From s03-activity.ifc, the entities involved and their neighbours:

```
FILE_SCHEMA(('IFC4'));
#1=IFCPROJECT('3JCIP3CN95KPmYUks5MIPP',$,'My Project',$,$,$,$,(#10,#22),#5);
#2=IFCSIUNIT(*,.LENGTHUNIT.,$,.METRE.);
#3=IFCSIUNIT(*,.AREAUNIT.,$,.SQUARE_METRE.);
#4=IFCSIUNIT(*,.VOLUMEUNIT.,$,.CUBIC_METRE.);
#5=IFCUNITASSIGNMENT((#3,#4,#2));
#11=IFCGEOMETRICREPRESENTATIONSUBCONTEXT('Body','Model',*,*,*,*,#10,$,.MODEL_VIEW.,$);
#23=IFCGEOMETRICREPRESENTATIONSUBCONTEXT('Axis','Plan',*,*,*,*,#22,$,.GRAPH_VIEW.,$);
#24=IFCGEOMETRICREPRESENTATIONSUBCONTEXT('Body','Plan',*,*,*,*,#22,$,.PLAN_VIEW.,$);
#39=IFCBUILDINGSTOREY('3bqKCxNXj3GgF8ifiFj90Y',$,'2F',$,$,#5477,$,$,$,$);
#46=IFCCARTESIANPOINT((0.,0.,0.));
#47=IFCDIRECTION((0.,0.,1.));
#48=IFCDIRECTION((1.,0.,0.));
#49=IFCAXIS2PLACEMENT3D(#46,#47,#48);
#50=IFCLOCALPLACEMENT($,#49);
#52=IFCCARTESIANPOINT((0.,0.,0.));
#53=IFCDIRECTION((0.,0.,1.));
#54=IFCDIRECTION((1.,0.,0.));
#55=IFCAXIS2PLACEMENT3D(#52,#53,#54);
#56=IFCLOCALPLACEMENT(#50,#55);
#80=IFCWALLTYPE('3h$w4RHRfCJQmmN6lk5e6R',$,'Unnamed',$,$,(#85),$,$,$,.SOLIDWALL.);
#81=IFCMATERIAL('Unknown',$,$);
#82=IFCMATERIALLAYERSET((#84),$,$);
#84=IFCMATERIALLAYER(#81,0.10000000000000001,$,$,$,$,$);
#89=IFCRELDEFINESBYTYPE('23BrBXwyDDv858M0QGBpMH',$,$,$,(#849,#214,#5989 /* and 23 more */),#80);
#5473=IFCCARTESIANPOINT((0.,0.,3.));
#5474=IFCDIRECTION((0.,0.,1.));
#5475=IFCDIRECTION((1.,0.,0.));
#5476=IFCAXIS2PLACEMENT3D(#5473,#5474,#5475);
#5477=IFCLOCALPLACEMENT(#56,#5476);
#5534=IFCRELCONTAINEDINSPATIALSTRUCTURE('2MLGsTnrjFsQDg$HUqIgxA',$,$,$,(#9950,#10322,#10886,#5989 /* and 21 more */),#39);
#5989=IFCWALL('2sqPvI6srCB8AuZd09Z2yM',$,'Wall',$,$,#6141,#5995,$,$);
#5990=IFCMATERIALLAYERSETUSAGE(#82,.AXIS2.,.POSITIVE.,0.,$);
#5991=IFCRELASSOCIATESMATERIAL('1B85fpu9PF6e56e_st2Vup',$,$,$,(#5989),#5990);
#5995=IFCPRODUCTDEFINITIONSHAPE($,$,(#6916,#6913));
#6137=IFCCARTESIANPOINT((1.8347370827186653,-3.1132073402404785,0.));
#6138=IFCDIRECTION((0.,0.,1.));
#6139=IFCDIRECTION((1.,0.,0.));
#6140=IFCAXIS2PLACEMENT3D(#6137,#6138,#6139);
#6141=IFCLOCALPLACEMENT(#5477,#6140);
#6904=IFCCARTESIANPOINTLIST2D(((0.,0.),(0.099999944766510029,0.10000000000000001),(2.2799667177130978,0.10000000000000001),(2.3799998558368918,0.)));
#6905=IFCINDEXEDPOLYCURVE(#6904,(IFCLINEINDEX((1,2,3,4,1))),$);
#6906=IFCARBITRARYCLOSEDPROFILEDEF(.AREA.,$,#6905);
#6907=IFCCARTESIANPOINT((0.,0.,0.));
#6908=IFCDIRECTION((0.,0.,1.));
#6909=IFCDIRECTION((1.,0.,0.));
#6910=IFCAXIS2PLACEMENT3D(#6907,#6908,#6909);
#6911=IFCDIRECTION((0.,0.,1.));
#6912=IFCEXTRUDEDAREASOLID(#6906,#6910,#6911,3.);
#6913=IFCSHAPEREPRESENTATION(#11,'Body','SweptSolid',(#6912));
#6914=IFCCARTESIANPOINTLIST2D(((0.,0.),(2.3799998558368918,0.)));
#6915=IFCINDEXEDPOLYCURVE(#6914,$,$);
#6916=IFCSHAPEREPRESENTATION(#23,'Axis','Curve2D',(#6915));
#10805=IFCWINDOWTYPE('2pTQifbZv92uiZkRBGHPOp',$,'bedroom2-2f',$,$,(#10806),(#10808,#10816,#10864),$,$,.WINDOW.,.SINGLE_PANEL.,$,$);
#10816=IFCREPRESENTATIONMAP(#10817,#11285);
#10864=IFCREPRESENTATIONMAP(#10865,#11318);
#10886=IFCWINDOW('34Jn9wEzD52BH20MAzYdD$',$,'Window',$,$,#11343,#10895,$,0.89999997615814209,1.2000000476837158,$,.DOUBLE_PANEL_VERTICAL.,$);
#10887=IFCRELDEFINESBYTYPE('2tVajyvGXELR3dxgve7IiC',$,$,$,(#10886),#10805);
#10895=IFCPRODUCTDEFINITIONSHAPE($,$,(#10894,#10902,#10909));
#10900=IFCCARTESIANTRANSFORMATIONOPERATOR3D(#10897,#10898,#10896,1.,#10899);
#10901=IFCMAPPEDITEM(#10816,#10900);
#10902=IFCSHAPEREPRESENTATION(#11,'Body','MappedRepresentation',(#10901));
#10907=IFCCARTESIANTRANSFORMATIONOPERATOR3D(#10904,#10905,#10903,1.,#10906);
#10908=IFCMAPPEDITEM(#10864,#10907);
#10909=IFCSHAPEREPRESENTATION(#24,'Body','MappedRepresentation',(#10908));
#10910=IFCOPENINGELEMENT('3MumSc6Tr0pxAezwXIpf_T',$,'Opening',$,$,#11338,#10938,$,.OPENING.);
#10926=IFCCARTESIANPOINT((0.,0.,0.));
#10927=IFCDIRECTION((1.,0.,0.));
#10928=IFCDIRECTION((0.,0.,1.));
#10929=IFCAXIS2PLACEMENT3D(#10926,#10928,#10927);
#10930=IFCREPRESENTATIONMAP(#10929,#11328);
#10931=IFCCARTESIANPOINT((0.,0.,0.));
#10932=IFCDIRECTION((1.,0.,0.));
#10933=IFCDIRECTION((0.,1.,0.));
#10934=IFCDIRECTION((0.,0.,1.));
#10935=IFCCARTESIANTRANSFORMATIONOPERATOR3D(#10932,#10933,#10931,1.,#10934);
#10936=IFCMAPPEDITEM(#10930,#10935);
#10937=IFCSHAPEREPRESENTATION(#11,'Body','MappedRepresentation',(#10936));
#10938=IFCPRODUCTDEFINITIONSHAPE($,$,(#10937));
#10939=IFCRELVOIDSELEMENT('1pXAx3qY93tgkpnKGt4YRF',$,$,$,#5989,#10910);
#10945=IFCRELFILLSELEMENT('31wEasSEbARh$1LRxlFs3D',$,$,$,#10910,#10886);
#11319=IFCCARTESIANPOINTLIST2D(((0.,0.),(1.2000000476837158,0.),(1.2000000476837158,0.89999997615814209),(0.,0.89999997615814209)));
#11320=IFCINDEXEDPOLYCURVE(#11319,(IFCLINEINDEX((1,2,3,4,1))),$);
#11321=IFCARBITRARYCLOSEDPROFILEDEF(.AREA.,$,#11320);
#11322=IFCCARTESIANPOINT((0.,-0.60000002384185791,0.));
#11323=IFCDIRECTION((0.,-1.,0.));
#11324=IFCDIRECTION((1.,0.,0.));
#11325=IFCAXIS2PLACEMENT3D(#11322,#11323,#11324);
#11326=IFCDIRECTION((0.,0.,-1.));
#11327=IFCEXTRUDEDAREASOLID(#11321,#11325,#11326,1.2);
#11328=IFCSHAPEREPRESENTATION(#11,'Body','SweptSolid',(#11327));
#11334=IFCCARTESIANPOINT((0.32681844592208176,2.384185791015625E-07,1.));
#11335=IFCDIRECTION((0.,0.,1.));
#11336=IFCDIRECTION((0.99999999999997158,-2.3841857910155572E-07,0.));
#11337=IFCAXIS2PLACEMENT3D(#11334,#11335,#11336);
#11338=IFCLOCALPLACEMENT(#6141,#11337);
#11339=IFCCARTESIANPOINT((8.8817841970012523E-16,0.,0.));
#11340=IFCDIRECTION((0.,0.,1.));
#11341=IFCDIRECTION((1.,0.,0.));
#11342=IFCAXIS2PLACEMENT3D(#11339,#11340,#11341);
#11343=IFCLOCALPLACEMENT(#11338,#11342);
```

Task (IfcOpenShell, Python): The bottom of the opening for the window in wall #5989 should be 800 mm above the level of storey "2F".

```python
import numpy as np
import ifcopenshell
import ifcopenshell.api.geometry
import ifcopenshell.geom
import ifcopenshell.util.element
import ifcopenshell.util.placement
import ifcopenshell.util.shape
import ifcopenshell.util.unit

model = ifcopenshell.open("s03-activity.ifc")
unit_scale = ifcopenshell.util.unit.calculate_unit_scale(model)

window = model.by_id(10886)
opening = window.FillsVoids[0].RelatingOpeningElement
storey = ifcopenshell.util.element.get_container(window, ifc_class="IfcBuildingStorey")
level = ifcopenshell.util.placement.get_local_placement(storey.ObjectPlacement)[2, 3]

# The opening's origin need not be at the sill, so measure its lowest point.
shape = ifcopenshell.geom.create_shape(ifcopenshell.geom.settings(), opening)
bottom = ifcopenshell.util.shape.get_shape_bottom_elevation(shape, shape.geometry) / unit_scale
dz = level + 0.8 / unit_scale - bottom

shift = np.array([0.0, 0.0, dz])
# The window is placed relative to its opening, so it follows when the opening moves.
matrix = ifcopenshell.util.placement.get_local_placement(opening.ObjectPlacement)
matrix[:3, 3] += shift
ifcopenshell.api.geometry.edit_object_placement(
    model, product=opening, matrix=matrix, is_si=False, should_transform_children=True
)

print(f"moved by {dz * unit_scale:+.3f} m")

model.write("s03-activity_rev.ifc")
```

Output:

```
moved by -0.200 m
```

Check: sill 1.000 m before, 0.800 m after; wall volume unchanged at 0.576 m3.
